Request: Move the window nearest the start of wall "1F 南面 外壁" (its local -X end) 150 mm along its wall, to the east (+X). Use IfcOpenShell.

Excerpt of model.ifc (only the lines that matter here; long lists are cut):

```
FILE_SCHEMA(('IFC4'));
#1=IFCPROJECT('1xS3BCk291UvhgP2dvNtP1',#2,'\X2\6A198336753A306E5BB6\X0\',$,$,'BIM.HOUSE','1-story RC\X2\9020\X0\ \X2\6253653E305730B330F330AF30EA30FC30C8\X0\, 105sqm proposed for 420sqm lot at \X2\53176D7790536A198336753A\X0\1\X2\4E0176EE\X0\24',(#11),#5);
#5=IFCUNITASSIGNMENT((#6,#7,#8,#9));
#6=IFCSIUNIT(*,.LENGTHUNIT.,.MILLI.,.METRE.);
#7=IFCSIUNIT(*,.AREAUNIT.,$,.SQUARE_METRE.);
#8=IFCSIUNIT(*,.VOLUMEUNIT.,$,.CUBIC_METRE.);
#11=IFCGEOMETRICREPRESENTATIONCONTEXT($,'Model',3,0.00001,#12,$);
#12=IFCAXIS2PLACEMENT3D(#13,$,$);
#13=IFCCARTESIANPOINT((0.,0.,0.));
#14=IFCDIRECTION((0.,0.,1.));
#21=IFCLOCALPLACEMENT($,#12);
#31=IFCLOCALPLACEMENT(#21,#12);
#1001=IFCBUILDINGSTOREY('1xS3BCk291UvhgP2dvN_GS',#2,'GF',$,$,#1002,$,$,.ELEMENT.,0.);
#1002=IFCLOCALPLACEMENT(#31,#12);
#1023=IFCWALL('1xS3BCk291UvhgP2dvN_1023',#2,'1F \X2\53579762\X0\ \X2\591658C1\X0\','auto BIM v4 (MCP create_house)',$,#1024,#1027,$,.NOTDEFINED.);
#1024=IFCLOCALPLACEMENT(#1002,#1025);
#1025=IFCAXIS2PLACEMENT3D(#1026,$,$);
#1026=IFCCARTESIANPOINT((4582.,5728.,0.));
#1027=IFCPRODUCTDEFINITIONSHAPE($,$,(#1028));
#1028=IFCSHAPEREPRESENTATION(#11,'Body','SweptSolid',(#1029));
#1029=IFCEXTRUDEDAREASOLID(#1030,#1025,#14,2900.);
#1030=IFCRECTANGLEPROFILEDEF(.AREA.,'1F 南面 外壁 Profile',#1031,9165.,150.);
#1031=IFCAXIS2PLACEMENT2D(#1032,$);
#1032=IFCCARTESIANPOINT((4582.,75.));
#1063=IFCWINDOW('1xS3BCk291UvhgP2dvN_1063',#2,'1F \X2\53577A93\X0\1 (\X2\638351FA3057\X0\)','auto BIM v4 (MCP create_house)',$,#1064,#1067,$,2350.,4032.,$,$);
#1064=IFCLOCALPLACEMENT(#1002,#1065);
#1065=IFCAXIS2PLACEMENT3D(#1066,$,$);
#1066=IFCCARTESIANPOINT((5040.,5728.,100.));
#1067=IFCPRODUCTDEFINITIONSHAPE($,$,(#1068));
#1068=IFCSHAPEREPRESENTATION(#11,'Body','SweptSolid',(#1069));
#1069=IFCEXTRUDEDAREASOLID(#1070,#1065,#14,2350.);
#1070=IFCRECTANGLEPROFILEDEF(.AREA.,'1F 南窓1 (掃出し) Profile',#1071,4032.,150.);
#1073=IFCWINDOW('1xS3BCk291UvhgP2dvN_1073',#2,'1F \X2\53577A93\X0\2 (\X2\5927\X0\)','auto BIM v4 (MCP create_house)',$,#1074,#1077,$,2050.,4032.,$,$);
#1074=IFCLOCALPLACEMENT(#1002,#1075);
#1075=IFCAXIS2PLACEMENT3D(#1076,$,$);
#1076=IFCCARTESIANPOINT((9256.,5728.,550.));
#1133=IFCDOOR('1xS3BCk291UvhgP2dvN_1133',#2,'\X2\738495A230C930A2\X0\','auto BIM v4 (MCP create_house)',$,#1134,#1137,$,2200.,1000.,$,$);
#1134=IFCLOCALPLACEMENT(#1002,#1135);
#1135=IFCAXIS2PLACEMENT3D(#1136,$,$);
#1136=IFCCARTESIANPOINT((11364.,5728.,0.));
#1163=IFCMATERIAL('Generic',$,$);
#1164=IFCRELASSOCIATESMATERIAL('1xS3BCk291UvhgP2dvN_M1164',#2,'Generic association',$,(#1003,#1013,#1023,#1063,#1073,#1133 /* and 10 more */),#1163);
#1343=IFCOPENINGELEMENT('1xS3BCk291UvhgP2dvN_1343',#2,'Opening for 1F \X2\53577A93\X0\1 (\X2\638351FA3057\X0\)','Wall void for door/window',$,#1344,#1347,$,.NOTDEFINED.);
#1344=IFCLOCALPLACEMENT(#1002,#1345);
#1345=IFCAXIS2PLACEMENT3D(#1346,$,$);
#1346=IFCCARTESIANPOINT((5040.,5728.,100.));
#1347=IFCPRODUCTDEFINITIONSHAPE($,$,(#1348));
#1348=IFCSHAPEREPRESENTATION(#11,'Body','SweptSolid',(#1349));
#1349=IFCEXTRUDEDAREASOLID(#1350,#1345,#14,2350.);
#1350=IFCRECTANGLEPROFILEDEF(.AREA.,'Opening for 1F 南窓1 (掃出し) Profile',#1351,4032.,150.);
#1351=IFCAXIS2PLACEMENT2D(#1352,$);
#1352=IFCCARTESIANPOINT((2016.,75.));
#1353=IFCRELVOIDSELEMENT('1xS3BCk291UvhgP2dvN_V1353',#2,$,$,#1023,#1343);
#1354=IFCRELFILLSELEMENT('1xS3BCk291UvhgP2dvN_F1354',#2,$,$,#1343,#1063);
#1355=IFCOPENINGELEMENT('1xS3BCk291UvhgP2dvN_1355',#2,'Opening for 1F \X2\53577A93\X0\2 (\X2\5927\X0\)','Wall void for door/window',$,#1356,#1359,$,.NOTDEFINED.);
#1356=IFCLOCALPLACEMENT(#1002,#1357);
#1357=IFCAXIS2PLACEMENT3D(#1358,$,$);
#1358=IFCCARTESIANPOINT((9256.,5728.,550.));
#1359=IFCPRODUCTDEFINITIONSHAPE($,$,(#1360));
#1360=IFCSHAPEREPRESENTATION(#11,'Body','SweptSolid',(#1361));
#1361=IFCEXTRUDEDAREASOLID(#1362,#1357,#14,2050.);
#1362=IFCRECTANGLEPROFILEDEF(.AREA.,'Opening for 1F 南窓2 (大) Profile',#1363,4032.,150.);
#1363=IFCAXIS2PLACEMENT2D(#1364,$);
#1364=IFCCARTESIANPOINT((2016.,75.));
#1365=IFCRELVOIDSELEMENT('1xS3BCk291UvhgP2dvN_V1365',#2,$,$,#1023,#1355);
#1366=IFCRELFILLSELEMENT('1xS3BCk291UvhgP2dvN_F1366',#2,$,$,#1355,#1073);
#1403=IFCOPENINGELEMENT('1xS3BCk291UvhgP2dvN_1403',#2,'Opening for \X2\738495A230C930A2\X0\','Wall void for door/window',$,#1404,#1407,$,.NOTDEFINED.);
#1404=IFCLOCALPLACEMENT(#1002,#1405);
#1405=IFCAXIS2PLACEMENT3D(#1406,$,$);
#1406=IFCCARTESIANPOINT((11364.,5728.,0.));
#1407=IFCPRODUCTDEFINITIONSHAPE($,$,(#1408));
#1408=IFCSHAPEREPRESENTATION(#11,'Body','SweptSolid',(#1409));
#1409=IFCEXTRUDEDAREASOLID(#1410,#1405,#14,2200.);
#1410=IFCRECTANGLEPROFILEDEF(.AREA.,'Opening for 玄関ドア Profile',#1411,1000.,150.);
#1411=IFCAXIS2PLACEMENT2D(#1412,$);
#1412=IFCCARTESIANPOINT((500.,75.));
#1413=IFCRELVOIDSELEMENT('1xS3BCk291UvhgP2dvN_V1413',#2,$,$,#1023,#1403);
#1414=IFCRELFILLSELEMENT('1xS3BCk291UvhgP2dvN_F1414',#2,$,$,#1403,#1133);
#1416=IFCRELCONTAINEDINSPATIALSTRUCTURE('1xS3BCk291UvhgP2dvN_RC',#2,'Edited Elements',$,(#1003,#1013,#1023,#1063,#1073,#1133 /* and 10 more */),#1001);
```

```python
import ifcopenshell
import ifcopenshell.api.geometry
import ifcopenshell.util.placement

model = ifcopenshell.open("model.ifc")

window = model.by_guid("1xS3BCk291UvhgP2dvN_1063")
opening = window.FillsVoids[0].RelatingOpeningElement
wall = opening.VoidsElements[0].RelatingBuildingElement

wall_matrix = ifcopenshell.util.placement.get_local_placement(wall.ObjectPlacement)
shift = wall_matrix[:3, 0] * 150.0
before = ifcopenshell.util.placement.get_local_placement(window.ObjectPlacement)[:3, 3].copy()

# The window is not placed relative to its opening, so move both.
for product in (opening, window):
    matrix = ifcopenshell.util.placement.get_local_placement(product.ObjectPlacement)
    matrix[:3, 3] += shift
    ifcopenshell.api.geometry.edit_object_placement(model, product=product, matrix=matrix, is_si=False)

after = ifcopenshell.util.placement.get_local_placement(window.ObjectPlacement)[:3, 3]
print("window moved by", (after - before).round(3) + 0.0)

model.write("model_updated.ifc")
```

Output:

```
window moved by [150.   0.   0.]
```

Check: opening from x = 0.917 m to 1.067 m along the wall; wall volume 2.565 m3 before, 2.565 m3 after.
